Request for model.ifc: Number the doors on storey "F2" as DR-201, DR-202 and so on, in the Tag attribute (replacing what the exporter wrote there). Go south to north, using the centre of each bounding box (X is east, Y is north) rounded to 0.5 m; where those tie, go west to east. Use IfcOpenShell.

First a look at what the model holds.

```python
import ifcopenshell
import ifcopenshell.util.element
import ifcopenshell.util.placement

model = ifcopenshell.open("model.ifc")
print(model.schema)
storey = next(s for s in model.by_type("IfcBuildingStorey") if s.Name == "F2")
doors = [e for e in ifcopenshell.util.element.get_decomposition(storey) if e.is_a("IfcDoor")]
for e in sorted(doors, key=lambda e: e.id()):
    origin = ifcopenshell.util.placement.get_local_placement(e.ObjectPlacement)[:3, 3]
    print(e.id(), e.Tag, e.Name, origin.round(2) + 0.0, sep=" | ")
```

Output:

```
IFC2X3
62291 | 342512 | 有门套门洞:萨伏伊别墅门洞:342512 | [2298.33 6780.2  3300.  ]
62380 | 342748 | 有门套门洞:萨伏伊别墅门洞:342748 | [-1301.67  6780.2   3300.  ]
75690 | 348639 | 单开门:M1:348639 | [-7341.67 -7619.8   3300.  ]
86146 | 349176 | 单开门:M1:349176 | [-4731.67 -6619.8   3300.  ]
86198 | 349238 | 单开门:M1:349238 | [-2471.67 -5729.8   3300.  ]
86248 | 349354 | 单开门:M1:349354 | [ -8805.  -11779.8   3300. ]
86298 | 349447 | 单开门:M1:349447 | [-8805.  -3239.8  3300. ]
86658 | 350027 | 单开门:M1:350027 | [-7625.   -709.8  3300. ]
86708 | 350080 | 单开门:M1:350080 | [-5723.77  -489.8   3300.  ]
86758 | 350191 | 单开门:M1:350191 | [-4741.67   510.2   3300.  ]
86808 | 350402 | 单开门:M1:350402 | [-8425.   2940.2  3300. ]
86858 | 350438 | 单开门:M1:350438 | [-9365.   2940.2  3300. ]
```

```python
import ifcopenshell
import ifcopenshell.geom
import ifcopenshell.util.element
import ifcopenshell.util.shape

model = ifcopenshell.open("model.ifc")
settings = ifcopenshell.geom.settings()
settings.set("use-world-coords", True)


def centre(element):
    shape = ifcopenshell.geom.create_shape(settings, element)
    return ifcopenshell.util.shape.get_bbox_centroid(shape.geometry)


storey = next(s for s in model.by_type("IfcBuildingStorey") if s.Name == "F2")
doors = [e for e in ifcopenshell.util.element.get_decomposition(storey) if e.is_a("IfcDoor")]

# Insertion points can sit at a corner or the storey origin, so sort by the geometry (in metres).
centres = {e: centre(e) for e in doors}
doors.sort(key=lambda e: (round(centres[e][1] / 0.5), centres[e][0]))

for i, e in enumerate(doors, start=1):
    number = f"DR-2{i:02d}"
    e.Tag = number
    print(e.id(), number)

model.write("model_edited.ifc")
```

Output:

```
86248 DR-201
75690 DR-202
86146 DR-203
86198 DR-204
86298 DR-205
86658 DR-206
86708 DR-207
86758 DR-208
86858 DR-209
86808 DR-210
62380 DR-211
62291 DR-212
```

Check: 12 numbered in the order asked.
